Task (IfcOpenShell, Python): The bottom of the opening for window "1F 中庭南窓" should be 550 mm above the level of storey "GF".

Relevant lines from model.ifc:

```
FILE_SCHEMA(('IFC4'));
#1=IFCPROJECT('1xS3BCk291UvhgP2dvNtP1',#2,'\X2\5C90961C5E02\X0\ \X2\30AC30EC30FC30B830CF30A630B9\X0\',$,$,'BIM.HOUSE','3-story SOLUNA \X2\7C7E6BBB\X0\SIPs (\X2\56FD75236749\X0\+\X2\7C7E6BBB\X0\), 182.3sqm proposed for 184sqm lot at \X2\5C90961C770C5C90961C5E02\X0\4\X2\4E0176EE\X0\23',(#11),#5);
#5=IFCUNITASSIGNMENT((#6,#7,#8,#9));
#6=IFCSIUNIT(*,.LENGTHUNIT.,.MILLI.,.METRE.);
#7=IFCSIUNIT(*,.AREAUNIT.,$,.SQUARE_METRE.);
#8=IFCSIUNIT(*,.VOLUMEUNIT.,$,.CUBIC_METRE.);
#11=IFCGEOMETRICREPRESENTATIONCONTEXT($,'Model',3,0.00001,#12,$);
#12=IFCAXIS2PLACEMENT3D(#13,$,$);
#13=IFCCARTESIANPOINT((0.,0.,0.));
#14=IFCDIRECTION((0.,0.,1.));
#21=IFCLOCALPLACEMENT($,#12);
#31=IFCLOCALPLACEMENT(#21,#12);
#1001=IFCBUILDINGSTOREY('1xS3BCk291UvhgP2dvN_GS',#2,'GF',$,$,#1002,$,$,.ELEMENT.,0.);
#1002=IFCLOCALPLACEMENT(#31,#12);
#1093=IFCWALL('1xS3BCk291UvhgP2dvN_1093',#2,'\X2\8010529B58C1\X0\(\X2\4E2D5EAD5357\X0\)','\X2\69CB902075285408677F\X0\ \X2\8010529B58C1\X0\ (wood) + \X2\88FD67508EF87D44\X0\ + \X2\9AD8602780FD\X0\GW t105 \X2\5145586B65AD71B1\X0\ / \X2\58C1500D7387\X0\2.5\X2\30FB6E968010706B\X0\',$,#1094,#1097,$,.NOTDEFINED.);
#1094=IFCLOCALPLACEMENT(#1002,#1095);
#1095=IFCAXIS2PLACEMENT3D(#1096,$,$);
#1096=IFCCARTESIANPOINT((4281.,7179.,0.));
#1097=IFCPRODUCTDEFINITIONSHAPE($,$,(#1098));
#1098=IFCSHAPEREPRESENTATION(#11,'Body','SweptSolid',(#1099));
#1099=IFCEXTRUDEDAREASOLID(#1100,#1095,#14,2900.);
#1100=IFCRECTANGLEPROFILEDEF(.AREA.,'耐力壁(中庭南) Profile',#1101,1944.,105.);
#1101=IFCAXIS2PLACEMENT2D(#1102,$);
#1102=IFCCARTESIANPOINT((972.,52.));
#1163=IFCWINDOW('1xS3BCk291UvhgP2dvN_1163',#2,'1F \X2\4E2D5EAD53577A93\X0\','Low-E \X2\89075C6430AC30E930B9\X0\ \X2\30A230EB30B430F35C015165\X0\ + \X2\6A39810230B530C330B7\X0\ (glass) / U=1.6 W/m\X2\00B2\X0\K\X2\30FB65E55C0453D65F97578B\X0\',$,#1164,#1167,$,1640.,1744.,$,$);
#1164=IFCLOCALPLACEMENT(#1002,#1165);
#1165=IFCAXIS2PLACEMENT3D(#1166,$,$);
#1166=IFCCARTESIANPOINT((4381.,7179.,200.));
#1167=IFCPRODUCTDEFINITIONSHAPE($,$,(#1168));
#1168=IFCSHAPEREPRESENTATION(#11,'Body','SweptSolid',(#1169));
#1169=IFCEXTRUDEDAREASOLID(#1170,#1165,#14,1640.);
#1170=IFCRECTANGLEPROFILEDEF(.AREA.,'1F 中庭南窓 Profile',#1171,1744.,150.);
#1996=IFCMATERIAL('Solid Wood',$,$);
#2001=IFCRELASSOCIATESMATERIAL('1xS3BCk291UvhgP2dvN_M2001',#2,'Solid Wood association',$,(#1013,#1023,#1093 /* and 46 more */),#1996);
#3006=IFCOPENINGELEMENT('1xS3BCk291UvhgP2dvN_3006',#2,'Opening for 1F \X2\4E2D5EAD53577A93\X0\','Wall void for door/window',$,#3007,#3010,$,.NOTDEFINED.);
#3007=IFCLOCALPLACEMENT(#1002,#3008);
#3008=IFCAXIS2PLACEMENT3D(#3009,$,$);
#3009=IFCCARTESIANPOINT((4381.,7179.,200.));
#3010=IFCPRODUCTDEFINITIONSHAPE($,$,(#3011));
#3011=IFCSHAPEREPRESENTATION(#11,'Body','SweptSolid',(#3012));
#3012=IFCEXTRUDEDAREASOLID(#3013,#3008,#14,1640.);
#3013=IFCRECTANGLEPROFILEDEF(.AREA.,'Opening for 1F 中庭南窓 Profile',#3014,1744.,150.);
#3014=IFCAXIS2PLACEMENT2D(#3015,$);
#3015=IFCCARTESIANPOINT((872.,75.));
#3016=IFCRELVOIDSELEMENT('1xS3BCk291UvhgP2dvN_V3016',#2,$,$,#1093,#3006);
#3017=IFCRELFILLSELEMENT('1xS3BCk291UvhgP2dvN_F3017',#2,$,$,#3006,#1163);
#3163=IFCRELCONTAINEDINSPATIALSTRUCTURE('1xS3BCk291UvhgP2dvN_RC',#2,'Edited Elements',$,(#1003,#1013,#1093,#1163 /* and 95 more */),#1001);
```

```python
import numpy as np
import ifcopenshell
import ifcopenshell.api.geometry
import ifcopenshell.geom
import ifcopenshell.util.element
import ifcopenshell.util.placement
import ifcopenshell.util.shape
import ifcopenshell.util.unit

model = ifcopenshell.open("model.ifc")
unit_scale = ifcopenshell.util.unit.calculate_unit_scale(model)

window = model.by_guid("1xS3BCk291UvhgP2dvN_1163")
opening = window.FillsVoids[0].RelatingOpeningElement
storey = ifcopenshell.util.element.get_container(window, ifc_class="IfcBuildingStorey")
level = ifcopenshell.util.placement.get_local_placement(storey.ObjectPlacement)[2, 3]

# The opening's origin need not be at the sill, so measure its lowest point.
shape = ifcopenshell.geom.create_shape(ifcopenshell.geom.settings(), opening)
bottom = ifcopenshell.util.shape.get_shape_bottom_elevation(shape, shape.geometry) / unit_scale
dz = level + 0.55 / unit_scale - bottom

shift = np.array([0.0, 0.0, dz])
# The window is not placed relative to its opening, so move both.
for product in (opening, window):
    matrix = ifcopenshell.util.placement.get_local_placement(product.ObjectPlacement)
    matrix[:3, 3] += shift
    ifcopenshell.api.geometry.edit_object_placement(model, product=product, matrix=matrix, is_si=False)

print(f"moved by {dz * unit_scale:+.3f} m")

model.write("model_rev.ifc")
```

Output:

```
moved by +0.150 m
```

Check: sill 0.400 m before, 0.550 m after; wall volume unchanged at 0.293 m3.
